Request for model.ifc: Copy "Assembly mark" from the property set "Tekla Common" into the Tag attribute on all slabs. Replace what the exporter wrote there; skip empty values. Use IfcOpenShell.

First a look at what the model holds.

```python
import ifcopenshell
import ifcopenshell.util.element

model = ifcopenshell.open("model.ifc")
print(model.schema)
slabs = model.by_type("IfcSlab")
print(len(slabs), "slabs")
for e in slabs[:8]:
    source = ifcopenshell.util.element.get_pset(e, "Tekla Common", "Assembly mark")
    target = e.Tag
    print(e.id(), repr(source), repr(target), sep=" | ")
```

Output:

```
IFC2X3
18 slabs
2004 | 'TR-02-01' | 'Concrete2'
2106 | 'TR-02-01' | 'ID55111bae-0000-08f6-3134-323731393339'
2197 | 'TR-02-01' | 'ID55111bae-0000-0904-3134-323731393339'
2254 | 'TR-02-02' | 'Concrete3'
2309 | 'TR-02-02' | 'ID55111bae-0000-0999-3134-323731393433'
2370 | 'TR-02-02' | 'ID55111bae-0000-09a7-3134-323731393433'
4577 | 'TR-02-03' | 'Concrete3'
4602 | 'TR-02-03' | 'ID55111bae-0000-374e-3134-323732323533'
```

```python
import ifcopenshell
import ifcopenshell.util.element

model = ifcopenshell.open("model.ifc")

count = 0
for e in model.by_type("IfcSlab"):
    value = ifcopenshell.util.element.get_pset(e, "Tekla Common", "Assembly mark")
    current = e.Tag
    if not value or not value.strip() or current == value:
        continue
    e.Tag = value
    count += 1

print(count, "slabs updated")

model.write("model_v2.ifc")
```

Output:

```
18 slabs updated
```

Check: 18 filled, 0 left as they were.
